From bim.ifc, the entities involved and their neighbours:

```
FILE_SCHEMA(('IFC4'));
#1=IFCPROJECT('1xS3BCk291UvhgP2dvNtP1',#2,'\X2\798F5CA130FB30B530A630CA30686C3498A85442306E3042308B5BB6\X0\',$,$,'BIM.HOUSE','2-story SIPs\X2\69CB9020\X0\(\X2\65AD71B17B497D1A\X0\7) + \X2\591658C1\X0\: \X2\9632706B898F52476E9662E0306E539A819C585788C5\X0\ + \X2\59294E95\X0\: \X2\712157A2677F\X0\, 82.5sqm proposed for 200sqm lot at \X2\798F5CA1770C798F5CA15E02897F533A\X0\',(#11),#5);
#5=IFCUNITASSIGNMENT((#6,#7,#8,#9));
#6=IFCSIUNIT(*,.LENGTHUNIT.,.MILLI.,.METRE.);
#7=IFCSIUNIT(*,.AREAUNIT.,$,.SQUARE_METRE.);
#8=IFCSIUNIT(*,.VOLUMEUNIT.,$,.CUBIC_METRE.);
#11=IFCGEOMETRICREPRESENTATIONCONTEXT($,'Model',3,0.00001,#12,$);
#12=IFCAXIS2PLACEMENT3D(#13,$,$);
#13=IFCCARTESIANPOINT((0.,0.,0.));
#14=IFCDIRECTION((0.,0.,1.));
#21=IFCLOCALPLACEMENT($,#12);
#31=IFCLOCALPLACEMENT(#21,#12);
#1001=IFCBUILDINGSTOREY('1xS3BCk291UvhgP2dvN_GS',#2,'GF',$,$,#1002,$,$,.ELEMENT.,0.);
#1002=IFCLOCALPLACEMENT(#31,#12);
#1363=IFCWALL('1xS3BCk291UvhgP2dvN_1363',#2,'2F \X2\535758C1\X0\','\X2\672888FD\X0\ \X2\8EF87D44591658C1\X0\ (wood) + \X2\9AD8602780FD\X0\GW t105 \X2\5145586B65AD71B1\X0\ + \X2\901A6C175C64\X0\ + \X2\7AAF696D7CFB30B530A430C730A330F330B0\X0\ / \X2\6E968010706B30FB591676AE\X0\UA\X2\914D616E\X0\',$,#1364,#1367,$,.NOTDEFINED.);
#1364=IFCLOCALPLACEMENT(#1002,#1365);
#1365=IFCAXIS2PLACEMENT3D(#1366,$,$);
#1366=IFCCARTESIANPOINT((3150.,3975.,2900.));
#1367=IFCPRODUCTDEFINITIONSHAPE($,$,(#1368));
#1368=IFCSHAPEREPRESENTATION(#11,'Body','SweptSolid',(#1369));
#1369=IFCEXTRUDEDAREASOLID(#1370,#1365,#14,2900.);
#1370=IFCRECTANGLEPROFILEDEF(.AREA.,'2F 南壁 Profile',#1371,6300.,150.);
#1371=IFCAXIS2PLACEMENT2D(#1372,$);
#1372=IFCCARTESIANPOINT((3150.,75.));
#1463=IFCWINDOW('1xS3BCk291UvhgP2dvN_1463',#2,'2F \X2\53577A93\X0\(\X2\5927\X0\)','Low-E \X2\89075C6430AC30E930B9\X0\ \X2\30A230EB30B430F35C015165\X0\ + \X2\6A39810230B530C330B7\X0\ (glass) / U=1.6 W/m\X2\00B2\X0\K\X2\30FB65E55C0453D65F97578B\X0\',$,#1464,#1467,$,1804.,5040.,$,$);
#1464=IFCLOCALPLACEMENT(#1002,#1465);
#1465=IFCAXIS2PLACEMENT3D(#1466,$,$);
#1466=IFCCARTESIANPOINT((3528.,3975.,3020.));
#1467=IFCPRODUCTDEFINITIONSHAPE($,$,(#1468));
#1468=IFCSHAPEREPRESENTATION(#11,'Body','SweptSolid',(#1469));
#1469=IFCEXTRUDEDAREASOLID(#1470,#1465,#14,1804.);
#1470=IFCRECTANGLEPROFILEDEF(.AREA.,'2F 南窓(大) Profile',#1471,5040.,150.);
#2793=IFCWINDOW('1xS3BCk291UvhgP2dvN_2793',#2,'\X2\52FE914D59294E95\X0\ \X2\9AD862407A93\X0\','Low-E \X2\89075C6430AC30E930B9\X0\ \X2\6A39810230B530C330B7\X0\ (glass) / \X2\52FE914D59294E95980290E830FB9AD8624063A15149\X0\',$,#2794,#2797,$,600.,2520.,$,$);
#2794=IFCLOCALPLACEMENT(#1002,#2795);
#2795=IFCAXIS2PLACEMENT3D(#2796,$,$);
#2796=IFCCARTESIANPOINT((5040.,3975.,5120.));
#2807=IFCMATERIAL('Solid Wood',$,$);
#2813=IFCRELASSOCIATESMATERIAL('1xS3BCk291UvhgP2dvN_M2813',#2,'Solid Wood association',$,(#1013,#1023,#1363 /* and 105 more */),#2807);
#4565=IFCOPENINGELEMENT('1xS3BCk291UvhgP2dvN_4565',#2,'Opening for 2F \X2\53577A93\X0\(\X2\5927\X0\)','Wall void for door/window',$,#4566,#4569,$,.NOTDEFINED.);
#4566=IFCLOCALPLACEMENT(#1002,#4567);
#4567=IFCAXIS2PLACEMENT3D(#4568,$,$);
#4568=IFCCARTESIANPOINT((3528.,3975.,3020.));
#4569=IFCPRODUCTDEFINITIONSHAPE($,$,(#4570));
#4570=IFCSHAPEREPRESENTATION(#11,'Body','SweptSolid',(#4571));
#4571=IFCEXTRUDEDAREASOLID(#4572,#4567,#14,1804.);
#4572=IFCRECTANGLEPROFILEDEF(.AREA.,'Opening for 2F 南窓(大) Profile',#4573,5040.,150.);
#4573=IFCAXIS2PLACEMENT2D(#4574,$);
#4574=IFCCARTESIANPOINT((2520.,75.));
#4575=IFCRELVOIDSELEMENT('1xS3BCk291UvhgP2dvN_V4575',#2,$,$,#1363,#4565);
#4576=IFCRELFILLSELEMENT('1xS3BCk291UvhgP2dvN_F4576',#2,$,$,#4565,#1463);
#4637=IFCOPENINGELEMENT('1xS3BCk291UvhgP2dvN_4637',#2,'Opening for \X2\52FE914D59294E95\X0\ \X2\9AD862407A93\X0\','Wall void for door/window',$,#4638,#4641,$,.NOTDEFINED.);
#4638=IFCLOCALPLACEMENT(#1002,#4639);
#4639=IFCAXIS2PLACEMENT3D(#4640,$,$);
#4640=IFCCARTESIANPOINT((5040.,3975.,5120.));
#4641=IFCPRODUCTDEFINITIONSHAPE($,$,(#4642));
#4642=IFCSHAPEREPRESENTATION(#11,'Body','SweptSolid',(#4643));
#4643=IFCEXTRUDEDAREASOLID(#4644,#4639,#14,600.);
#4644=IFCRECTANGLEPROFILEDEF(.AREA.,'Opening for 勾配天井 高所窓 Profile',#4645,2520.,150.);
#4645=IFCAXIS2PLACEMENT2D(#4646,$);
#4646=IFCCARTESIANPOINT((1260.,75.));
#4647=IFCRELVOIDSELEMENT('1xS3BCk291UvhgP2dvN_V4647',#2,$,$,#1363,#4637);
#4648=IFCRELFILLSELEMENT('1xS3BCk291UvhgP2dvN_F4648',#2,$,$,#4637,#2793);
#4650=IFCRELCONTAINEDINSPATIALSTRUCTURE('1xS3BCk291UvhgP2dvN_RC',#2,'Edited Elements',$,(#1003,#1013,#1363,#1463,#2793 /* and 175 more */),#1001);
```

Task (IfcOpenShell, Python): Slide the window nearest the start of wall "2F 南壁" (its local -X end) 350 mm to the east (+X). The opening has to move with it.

```python
import ifcopenshell
import ifcopenshell.api.geometry
import ifcopenshell.util.placement
import ifcopenshell.util.unit

model = ifcopenshell.open("bim.ifc")
unit_scale = ifcopenshell.util.unit.calculate_unit_scale(model)

window = model.by_id(1463)
opening = window.FillsVoids[0].RelatingOpeningElement
wall = opening.VoidsElements[0].RelatingBuildingElement

wall_matrix = ifcopenshell.util.placement.get_local_placement(wall.ObjectPlacement)
shift = wall_matrix[:3, 0] * 0.35 / unit_scale
before = ifcopenshell.util.placement.get_local_placement(window.ObjectPlacement)[:3, 3].copy()

# The window is not placed relative to its opening, so move both.
for product in (opening, window):
    matrix = ifcopenshell.util.placement.get_local_placement(product.ObjectPlacement)
    matrix[:3, 3] += shift
    ifcopenshell.api.geometry.edit_object_placement(model, product=product, matrix=matrix, is_si=False)

after = ifcopenshell.util.placement.get_local_placement(window.ObjectPlacement)[:3, 3]
print("window moved by", (after - before).round(3) + 0.0)

model.write("bim-out.ifc")
```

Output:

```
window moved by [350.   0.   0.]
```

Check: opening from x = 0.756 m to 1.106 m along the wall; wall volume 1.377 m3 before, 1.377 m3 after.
